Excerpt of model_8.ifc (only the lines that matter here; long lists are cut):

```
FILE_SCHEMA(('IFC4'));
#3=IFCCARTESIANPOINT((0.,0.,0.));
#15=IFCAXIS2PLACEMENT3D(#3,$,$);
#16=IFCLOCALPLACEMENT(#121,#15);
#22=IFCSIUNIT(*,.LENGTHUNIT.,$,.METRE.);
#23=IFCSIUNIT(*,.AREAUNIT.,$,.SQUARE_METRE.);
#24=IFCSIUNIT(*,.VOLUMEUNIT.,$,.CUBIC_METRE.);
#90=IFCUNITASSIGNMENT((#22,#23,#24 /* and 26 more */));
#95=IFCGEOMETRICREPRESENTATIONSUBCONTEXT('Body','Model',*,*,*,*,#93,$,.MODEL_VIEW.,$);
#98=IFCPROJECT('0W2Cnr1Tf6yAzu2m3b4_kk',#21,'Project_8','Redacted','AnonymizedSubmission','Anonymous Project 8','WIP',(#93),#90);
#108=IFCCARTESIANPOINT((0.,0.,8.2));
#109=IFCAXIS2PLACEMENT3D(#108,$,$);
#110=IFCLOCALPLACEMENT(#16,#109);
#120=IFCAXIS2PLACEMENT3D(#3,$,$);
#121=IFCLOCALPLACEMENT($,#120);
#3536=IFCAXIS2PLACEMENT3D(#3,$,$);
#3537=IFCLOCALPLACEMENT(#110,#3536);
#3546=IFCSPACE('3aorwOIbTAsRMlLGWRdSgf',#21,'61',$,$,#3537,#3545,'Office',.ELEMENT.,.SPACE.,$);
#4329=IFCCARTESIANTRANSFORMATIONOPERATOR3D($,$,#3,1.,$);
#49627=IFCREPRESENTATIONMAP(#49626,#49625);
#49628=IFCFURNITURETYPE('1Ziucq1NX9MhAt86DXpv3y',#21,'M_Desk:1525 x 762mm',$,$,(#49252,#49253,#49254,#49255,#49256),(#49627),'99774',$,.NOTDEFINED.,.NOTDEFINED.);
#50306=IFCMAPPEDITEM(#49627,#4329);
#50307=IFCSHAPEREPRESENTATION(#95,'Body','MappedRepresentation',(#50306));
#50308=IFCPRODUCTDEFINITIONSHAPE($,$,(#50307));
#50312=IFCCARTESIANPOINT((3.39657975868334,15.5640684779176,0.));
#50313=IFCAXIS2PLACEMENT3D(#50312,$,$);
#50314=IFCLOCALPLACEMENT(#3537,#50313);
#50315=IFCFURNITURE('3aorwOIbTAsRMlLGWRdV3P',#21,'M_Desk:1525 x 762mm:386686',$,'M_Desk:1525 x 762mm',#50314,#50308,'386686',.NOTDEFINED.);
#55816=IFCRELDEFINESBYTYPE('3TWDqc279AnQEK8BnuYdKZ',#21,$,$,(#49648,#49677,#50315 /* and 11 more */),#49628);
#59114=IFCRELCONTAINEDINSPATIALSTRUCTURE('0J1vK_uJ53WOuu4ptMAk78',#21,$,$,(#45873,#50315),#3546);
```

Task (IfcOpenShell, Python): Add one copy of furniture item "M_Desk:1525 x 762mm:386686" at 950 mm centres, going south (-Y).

```python
import numpy as np
import ifcopenshell
import ifcopenshell.api.geometry
import ifcopenshell.api.root
import ifcopenshell.util.element
import ifcopenshell.util.placement
import ifcopenshell.util.unit

model = ifcopenshell.open("model_8.ifc")
unit_scale = ifcopenshell.util.unit.calculate_unit_scale(model)


def reuse_history(source, copy):
    """copy_class also copies each property set's owner history, people and application; keep the originals."""
    for rel in copy.IsDefinedBy:
        if rel.is_a("IfcRelDefinesByProperties") and (history := rel.RelatingPropertyDefinition.OwnerHistory):
            rel.RelatingPropertyDefinition.OwnerHistory = source.OwnerHistory
            ifcopenshell.util.element.remove_deep2(model, history)


source = model.by_guid("3aorwOIbTAsRMlLGWRdV3P")
base = ifcopenshell.util.placement.get_local_placement(source.ObjectPlacement)
step = np.array([0.0, -1.0, 0.0]) * 0.95 / unit_scale

for i in range(1, 2):
    copy = ifcopenshell.api.root.copy_class(model, product=source)
    copy.Representation = ifcopenshell.util.element.copy_deep(
        model, source.Representation, exclude=["IfcGeometricRepresentationContext", "IfcRepresentationMap"]
    )
    copy.Name = "M_Desk:1525 x 762mm"
    copy.Tag = None
    reuse_history(source, copy)
    matrix = base.copy()
    matrix[:3, 3] += i * step
    print("added at", matrix[:3, 3].round(3) + 0.0)
    ifcopenshell.api.geometry.edit_object_placement(model, product=copy, matrix=matrix, is_si=False)

model.write("model_8_v2.ifc")
```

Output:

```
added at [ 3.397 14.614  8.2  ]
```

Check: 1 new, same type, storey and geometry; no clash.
